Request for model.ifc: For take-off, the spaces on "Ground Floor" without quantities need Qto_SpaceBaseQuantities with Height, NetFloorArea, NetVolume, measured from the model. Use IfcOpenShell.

First a look at what the model holds.

```python
import ifcopenshell
import ifcopenshell.util.element
import ifcopenshell.util.unit

model = ifcopenshell.open("model.ifc")
print(model.schema)
for unit_type in ("LENGTHUNIT", "AREAUNIT", "VOLUMEUNIT"):
    print(unit_type, ifcopenshell.util.unit.calculate_unit_scale(model, unit_type))
storey = next(s for s in model.by_type("IfcBuildingStorey") if s.Name == "Ground Floor")
spaces = [e for e in ifcopenshell.util.element.get_decomposition(storey) if e.is_a("IfcSpace")]
for e in sorted(spaces, key=lambda e: e.id()):
    print(e.id(), e.is_a(), e.Name, list(ifcopenshell.util.element.get_psets(e, qtos_only=True)), sep=" | ")
```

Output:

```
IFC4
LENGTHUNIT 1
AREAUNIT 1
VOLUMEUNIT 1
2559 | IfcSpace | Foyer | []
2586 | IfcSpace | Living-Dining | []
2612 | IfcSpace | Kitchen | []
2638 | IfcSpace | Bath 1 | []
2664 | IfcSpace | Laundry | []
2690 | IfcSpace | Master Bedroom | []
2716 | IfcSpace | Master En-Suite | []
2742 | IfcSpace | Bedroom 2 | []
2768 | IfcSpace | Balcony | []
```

```python
import ifcopenshell
import ifcopenshell.api.pset
import ifcopenshell.geom
import ifcopenshell.util.element
import ifcopenshell.util.shape
import ifcopenshell.util.unit

model = ifcopenshell.open("model.ifc")
unit_scale = ifcopenshell.util.unit.calculate_unit_scale(model)
area_scale = ifcopenshell.util.unit.calculate_unit_scale(model, "AREAUNIT")
volume_scale = ifcopenshell.util.unit.calculate_unit_scale(model, "VOLUMEUNIT")
settings = ifcopenshell.geom.settings()

storey = next(s for s in model.by_type("IfcBuildingStorey") if s.Name == "Ground Floor")
spaces = [e for e in ifcopenshell.util.element.get_decomposition(storey) if e.is_a("IfcSpace")]

for e in sorted(spaces, key=lambda e: e.id()):
    if ifcopenshell.util.element.get_psets(e, qtos_only=True, should_inherit=False):
        continue
    # Geometry comes back in metres, in the element's own axes.
    shape = ifcopenshell.geom.create_shape(settings, e)
    values = {
        "Height": ifcopenshell.util.shape.get_z(shape.geometry) / unit_scale,
        "NetFloorArea": ifcopenshell.util.shape.get_footprint_area(shape.geometry) / area_scale,
        "NetVolume": ifcopenshell.util.shape.get_volume(shape.geometry) / volume_scale,
    }
    qto = ifcopenshell.api.pset.add_qto(model, product=e, name="Qto_SpaceBaseQuantities")
    ifcopenshell.api.pset.edit_qto(model, qto=qto, properties=values)
    print(e.id(), {k: round(v, 3) for k, v in values.items()})

model.write("model_updated.ifc")
```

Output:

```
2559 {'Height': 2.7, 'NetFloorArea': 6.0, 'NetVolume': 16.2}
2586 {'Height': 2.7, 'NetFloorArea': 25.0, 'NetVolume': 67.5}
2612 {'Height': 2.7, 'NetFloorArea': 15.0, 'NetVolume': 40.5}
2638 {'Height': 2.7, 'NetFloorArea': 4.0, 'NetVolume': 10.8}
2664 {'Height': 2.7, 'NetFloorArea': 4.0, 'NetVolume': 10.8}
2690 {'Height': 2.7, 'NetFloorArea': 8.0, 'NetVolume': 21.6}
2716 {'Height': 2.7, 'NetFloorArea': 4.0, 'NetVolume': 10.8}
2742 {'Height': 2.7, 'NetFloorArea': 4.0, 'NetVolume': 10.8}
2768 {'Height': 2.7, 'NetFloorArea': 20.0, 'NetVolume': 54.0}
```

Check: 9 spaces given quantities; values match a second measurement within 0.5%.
